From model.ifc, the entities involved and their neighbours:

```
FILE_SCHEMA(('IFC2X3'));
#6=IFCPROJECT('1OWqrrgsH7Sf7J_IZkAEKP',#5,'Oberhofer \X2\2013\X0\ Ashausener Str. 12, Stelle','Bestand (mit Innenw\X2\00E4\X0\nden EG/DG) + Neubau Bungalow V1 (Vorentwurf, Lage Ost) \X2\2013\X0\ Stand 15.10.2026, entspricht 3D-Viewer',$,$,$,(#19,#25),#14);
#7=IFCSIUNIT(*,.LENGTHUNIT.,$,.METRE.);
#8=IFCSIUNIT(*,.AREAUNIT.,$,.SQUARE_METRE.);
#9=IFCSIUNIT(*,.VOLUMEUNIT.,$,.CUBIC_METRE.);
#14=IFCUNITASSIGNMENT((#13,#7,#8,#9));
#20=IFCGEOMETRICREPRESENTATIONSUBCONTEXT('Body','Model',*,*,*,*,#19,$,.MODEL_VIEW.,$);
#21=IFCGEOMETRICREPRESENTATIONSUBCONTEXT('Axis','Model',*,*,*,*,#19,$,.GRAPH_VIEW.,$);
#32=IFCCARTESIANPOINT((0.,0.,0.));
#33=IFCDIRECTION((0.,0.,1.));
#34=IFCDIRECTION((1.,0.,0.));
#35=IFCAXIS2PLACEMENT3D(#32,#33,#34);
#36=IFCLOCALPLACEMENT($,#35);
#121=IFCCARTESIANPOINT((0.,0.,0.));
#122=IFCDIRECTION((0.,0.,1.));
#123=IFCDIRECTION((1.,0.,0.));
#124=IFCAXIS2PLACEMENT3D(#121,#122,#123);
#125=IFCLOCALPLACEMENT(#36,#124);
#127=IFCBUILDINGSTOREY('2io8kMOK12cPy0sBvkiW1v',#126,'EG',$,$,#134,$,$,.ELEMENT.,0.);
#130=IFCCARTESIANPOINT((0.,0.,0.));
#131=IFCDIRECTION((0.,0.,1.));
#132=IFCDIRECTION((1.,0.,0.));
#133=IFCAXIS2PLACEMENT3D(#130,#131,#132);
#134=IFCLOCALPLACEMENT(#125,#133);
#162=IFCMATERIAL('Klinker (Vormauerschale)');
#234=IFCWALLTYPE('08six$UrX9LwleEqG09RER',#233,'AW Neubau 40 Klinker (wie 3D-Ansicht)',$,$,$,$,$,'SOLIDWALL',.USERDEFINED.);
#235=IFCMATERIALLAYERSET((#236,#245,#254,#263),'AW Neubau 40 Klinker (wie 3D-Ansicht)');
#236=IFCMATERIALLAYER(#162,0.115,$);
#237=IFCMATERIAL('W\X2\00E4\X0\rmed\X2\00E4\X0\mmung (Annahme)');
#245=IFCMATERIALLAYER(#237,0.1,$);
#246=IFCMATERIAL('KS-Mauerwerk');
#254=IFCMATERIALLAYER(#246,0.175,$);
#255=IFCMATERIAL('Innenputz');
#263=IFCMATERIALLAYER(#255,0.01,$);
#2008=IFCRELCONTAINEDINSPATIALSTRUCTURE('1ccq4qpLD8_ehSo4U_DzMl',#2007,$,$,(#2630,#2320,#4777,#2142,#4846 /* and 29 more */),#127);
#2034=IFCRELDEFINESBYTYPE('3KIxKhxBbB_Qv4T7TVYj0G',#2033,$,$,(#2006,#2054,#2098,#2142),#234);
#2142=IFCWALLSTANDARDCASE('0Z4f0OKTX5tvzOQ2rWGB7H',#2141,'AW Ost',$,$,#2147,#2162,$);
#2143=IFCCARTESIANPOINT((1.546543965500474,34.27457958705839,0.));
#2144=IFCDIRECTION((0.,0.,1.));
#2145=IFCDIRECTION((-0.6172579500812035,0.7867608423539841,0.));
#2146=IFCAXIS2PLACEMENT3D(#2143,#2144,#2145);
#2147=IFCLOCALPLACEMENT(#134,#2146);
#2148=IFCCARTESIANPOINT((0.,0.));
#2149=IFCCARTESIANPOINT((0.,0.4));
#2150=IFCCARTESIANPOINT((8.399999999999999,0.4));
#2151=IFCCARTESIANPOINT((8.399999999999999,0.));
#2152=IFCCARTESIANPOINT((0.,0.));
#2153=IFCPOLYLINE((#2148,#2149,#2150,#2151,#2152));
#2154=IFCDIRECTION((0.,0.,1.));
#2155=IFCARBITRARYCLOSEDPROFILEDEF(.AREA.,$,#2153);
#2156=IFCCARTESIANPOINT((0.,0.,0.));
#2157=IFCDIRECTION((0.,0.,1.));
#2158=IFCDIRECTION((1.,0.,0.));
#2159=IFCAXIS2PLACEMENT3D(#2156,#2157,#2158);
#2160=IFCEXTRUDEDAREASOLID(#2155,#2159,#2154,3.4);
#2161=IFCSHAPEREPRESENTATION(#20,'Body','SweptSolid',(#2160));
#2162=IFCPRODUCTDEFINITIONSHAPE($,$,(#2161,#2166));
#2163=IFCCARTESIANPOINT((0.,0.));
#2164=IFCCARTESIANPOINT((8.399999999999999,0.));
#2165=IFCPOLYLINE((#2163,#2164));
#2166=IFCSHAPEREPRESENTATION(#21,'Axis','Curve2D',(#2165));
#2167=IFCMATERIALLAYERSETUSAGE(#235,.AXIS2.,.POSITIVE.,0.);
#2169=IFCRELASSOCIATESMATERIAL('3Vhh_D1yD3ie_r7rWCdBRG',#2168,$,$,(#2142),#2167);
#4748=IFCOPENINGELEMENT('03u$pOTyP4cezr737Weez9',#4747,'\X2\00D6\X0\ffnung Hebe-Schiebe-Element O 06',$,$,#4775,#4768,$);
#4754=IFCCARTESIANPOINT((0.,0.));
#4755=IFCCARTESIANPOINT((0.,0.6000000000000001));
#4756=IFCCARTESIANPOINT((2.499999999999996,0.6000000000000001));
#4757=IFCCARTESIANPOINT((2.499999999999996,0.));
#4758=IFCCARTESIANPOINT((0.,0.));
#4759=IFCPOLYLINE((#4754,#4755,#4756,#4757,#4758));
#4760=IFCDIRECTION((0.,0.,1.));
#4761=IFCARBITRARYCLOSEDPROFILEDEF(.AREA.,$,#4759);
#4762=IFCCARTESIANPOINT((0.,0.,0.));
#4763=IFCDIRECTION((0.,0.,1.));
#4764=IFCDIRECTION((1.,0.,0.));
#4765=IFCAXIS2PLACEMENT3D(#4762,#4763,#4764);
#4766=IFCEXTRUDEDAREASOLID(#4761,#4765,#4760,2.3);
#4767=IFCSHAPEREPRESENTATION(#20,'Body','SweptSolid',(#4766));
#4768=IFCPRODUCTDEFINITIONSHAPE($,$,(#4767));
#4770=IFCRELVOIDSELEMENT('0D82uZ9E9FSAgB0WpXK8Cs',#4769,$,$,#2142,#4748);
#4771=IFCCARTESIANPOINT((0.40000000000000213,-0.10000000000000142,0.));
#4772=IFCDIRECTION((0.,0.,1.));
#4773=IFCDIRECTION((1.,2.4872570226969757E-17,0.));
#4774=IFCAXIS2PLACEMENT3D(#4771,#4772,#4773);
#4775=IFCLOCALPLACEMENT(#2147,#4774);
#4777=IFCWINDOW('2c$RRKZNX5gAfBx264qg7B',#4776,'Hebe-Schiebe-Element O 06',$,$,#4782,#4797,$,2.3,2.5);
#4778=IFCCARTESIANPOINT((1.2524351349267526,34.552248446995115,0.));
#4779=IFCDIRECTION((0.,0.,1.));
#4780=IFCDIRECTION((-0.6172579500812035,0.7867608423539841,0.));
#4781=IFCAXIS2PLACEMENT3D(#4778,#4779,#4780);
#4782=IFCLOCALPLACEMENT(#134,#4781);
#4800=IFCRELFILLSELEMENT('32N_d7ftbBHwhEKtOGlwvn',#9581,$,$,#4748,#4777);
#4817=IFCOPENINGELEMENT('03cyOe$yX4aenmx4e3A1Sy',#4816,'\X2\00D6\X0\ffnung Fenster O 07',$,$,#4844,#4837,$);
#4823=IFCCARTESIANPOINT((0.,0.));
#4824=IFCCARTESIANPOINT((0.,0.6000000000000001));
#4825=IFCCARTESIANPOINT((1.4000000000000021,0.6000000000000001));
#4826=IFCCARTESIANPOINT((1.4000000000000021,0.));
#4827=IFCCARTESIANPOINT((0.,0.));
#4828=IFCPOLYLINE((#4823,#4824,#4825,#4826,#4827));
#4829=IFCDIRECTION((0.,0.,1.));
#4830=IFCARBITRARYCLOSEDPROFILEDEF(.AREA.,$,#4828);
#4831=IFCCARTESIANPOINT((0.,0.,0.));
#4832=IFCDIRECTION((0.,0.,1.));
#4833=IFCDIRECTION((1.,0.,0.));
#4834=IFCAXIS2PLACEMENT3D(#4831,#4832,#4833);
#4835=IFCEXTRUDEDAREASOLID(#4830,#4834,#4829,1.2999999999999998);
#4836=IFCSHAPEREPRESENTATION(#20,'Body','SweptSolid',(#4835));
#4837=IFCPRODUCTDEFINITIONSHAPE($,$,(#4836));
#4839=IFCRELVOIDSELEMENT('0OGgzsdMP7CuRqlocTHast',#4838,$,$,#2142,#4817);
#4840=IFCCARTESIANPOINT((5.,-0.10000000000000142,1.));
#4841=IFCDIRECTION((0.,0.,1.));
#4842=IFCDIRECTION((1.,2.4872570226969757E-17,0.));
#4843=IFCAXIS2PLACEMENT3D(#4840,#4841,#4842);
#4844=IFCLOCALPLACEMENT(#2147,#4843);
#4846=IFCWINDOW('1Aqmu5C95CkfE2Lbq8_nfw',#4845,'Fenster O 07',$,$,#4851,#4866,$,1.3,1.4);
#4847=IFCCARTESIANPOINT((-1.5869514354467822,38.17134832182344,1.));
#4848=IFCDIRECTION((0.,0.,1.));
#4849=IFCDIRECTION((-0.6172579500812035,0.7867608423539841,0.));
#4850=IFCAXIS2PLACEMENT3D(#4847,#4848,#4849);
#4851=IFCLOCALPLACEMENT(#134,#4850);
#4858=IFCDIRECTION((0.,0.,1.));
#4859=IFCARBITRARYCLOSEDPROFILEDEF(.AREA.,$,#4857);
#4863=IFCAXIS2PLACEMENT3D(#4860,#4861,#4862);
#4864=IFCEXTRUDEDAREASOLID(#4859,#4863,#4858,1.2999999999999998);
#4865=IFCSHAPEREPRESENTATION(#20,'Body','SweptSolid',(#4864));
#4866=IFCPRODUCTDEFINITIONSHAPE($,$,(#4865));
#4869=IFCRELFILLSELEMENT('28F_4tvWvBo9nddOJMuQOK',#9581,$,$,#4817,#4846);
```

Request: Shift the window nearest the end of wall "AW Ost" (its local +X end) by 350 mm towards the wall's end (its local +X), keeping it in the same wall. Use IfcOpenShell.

```python
import ifcopenshell
import ifcopenshell.api.geometry
import ifcopenshell.util.placement
import ifcopenshell.util.unit

model = ifcopenshell.open("model.ifc")
unit_scale = ifcopenshell.util.unit.calculate_unit_scale(model)

window = model.by_guid("1Aqmu5C95CkfE2Lbq8_nfw")
opening = window.FillsVoids[0].RelatingOpeningElement
wall = opening.VoidsElements[0].RelatingBuildingElement

wall_matrix = ifcopenshell.util.placement.get_local_placement(wall.ObjectPlacement)
shift = wall_matrix[:3, 0] * 0.35 / unit_scale
before = ifcopenshell.util.placement.get_local_placement(window.ObjectPlacement)[:3, 3].copy()

# The window is not placed relative to its opening, so move both.
for product in (opening, window):
    matrix = ifcopenshell.util.placement.get_local_placement(product.ObjectPlacement)
    matrix[:3, 3] += shift
    ifcopenshell.api.geometry.edit_object_placement(model, product=product, matrix=matrix, is_si=False)

after = ifcopenshell.util.placement.get_local_placement(window.ObjectPlacement)[:3, 3]
print("window moved by", (after - before).round(3) + 0.0)

model.write("model_v2.ifc")
```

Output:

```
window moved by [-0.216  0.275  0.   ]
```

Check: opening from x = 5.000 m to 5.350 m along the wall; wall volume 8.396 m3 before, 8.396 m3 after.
